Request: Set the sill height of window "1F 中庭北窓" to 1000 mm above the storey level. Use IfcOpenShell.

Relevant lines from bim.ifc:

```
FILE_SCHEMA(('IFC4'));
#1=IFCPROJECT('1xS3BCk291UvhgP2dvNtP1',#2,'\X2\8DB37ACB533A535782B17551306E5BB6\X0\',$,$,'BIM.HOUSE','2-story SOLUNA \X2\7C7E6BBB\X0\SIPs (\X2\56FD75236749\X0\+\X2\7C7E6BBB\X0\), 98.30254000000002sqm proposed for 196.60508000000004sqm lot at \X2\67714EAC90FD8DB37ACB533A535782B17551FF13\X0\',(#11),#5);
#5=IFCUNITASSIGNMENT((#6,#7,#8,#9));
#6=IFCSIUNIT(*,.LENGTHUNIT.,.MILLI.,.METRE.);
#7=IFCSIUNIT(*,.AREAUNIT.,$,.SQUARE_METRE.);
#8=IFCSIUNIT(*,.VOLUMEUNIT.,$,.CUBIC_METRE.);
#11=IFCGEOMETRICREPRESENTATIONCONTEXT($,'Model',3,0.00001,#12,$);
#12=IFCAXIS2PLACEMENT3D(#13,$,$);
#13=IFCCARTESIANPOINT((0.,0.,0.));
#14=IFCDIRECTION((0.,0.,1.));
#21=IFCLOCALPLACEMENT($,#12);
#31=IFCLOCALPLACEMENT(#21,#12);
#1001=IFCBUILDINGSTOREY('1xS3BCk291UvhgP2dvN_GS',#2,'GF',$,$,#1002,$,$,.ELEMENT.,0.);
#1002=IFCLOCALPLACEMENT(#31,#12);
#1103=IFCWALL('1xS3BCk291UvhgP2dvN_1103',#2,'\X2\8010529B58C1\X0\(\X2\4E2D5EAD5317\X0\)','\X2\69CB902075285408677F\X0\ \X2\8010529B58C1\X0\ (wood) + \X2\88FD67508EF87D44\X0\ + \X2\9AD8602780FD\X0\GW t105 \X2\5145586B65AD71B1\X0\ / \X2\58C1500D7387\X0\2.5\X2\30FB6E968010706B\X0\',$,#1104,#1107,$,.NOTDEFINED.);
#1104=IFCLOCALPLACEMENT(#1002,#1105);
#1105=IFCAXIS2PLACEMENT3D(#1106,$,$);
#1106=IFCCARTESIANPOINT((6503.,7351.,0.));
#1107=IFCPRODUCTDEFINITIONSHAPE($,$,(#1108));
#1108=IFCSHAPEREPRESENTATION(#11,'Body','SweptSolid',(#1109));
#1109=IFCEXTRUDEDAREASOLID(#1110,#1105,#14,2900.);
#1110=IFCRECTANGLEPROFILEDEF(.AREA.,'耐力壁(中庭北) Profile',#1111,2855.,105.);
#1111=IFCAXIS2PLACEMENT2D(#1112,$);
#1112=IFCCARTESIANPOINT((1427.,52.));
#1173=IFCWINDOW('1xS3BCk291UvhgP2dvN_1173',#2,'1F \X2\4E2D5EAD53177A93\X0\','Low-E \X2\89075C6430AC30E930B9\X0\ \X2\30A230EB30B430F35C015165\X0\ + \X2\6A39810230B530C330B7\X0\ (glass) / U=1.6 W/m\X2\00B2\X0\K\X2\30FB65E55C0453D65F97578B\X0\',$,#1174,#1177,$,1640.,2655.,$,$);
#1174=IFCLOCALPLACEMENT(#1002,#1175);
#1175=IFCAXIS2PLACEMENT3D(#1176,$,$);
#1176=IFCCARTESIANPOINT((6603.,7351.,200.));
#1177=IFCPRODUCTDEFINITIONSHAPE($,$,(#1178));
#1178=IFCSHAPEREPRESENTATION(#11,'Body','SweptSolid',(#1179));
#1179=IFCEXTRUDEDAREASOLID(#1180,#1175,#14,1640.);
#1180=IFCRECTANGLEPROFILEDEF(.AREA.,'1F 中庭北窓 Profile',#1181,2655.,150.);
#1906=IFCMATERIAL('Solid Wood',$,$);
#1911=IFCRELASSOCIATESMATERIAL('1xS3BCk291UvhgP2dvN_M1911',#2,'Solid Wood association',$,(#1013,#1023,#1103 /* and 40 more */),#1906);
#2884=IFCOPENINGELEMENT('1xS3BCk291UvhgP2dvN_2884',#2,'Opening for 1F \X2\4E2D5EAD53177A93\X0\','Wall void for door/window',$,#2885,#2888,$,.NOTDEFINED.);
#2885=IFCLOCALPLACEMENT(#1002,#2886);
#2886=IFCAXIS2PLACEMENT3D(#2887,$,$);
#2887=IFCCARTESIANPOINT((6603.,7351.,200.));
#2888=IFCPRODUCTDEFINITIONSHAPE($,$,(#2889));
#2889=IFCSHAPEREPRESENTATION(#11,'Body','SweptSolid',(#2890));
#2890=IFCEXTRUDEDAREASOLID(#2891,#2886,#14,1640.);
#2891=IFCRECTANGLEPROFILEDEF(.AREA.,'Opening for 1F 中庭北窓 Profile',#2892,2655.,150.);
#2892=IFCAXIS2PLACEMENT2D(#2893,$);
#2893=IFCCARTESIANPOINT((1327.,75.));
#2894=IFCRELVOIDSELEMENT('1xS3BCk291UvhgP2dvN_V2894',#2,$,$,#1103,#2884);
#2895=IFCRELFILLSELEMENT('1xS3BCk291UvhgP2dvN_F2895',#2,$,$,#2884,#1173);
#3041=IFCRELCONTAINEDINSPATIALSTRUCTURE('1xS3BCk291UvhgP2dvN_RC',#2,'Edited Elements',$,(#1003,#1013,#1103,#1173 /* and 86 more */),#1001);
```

```python
import numpy as np
import ifcopenshell
import ifcopenshell.api.geometry
import ifcopenshell.geom
import ifcopenshell.util.element
import ifcopenshell.util.placement
import ifcopenshell.util.shape
import ifcopenshell.util.unit

model = ifcopenshell.open("bim.ifc")
unit_scale = ifcopenshell.util.unit.calculate_unit_scale(model)

window = model.by_guid("1xS3BCk291UvhgP2dvN_1173")
opening = window.FillsVoids[0].RelatingOpeningElement
storey = ifcopenshell.util.element.get_container(window, ifc_class="IfcBuildingStorey")
level = ifcopenshell.util.placement.get_local_placement(storey.ObjectPlacement)[2, 3]

# The opening's origin need not be at the sill, so measure its lowest point.
shape = ifcopenshell.geom.create_shape(ifcopenshell.geom.settings(), opening)
bottom = ifcopenshell.util.shape.get_shape_bottom_elevation(shape, shape.geometry) / unit_scale
dz = level + 1 / unit_scale - bottom

shift = np.array([0.0, 0.0, dz])
# The window is not placed relative to its opening, so move both.
for product in (opening, window):
    matrix = ifcopenshell.util.placement.get_local_placement(product.ObjectPlacement)
    matrix[:3, 3] += shift
    ifcopenshell.api.geometry.edit_object_placement(model, product=product, matrix=matrix, is_si=False)

print(f"moved by {dz * unit_scale:+.3f} m")

model.write("bim_rev.ifc")
```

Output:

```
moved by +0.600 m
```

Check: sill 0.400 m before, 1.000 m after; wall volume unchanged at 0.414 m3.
